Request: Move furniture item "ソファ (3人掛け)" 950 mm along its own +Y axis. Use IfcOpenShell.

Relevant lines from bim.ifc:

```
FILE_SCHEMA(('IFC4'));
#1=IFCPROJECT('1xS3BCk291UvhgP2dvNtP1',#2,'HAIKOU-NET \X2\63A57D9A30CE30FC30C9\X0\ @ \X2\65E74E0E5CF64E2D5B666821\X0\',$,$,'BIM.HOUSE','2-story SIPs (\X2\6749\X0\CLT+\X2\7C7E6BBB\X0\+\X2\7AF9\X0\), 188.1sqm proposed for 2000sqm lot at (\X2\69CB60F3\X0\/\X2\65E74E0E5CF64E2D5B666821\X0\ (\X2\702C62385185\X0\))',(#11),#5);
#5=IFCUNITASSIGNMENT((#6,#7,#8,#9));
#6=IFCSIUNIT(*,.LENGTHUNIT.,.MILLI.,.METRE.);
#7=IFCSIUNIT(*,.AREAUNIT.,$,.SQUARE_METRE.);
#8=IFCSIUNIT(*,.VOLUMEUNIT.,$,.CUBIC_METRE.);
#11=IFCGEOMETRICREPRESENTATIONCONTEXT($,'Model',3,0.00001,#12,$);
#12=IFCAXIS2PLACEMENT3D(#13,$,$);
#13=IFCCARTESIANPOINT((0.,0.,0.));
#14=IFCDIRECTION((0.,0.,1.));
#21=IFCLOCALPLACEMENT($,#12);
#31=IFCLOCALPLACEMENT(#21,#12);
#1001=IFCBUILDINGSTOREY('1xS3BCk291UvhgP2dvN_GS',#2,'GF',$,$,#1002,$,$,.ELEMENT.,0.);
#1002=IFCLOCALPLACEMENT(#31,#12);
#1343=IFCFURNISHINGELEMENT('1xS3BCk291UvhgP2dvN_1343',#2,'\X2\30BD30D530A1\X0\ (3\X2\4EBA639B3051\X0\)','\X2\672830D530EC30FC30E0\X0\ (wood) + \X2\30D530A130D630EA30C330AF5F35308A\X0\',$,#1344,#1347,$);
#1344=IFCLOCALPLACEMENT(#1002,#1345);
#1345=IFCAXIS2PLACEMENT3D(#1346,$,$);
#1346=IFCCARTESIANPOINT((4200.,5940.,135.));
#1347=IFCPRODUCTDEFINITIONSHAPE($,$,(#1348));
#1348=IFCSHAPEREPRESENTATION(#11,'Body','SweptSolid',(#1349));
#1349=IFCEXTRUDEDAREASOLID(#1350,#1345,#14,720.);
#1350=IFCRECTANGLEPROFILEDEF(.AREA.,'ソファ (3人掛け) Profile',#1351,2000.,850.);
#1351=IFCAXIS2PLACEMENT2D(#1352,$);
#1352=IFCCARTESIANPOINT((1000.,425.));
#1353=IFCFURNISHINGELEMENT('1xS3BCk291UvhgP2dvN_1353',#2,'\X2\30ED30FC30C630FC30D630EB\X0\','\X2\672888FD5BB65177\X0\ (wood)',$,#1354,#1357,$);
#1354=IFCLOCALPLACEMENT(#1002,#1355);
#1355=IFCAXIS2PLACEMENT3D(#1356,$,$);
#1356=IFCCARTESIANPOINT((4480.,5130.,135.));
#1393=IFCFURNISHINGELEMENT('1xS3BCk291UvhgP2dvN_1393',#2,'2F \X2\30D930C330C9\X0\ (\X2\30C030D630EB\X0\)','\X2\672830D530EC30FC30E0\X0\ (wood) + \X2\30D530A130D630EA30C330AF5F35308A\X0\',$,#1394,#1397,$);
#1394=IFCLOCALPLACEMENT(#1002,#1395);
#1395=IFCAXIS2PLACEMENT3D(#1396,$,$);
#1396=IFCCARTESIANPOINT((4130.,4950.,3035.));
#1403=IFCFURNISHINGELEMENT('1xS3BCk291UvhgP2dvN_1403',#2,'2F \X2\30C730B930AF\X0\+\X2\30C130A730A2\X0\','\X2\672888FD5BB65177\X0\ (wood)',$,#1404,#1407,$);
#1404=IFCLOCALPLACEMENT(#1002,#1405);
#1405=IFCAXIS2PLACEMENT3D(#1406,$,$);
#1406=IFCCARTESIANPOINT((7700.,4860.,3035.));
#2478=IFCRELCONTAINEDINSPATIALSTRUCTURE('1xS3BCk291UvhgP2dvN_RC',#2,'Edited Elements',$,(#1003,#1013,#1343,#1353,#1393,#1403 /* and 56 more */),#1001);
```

```python
import ifcopenshell
import ifcopenshell.api.geometry
import ifcopenshell.util.placement
import ifcopenshell.util.unit

model = ifcopenshell.open("bim.ifc")
unit_scale = ifcopenshell.util.unit.calculate_unit_scale(model)

item = model.by_id(1343)
matrix = ifcopenshell.util.placement.get_local_placement(item.ObjectPlacement)
matrix[:3, 3] += matrix[:3, 1] * 0.95 / unit_scale
ifcopenshell.api.geometry.edit_object_placement(model, product=item, matrix=matrix, is_si=False)

print(ifcopenshell.util.placement.get_local_placement(item.ObjectPlacement).round(3) + 0.0)

model.write("bim_edited.ifc")
```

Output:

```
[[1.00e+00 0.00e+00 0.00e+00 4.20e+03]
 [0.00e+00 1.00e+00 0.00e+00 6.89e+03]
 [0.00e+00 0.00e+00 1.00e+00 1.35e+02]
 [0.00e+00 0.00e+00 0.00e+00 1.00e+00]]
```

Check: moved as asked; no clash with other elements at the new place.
